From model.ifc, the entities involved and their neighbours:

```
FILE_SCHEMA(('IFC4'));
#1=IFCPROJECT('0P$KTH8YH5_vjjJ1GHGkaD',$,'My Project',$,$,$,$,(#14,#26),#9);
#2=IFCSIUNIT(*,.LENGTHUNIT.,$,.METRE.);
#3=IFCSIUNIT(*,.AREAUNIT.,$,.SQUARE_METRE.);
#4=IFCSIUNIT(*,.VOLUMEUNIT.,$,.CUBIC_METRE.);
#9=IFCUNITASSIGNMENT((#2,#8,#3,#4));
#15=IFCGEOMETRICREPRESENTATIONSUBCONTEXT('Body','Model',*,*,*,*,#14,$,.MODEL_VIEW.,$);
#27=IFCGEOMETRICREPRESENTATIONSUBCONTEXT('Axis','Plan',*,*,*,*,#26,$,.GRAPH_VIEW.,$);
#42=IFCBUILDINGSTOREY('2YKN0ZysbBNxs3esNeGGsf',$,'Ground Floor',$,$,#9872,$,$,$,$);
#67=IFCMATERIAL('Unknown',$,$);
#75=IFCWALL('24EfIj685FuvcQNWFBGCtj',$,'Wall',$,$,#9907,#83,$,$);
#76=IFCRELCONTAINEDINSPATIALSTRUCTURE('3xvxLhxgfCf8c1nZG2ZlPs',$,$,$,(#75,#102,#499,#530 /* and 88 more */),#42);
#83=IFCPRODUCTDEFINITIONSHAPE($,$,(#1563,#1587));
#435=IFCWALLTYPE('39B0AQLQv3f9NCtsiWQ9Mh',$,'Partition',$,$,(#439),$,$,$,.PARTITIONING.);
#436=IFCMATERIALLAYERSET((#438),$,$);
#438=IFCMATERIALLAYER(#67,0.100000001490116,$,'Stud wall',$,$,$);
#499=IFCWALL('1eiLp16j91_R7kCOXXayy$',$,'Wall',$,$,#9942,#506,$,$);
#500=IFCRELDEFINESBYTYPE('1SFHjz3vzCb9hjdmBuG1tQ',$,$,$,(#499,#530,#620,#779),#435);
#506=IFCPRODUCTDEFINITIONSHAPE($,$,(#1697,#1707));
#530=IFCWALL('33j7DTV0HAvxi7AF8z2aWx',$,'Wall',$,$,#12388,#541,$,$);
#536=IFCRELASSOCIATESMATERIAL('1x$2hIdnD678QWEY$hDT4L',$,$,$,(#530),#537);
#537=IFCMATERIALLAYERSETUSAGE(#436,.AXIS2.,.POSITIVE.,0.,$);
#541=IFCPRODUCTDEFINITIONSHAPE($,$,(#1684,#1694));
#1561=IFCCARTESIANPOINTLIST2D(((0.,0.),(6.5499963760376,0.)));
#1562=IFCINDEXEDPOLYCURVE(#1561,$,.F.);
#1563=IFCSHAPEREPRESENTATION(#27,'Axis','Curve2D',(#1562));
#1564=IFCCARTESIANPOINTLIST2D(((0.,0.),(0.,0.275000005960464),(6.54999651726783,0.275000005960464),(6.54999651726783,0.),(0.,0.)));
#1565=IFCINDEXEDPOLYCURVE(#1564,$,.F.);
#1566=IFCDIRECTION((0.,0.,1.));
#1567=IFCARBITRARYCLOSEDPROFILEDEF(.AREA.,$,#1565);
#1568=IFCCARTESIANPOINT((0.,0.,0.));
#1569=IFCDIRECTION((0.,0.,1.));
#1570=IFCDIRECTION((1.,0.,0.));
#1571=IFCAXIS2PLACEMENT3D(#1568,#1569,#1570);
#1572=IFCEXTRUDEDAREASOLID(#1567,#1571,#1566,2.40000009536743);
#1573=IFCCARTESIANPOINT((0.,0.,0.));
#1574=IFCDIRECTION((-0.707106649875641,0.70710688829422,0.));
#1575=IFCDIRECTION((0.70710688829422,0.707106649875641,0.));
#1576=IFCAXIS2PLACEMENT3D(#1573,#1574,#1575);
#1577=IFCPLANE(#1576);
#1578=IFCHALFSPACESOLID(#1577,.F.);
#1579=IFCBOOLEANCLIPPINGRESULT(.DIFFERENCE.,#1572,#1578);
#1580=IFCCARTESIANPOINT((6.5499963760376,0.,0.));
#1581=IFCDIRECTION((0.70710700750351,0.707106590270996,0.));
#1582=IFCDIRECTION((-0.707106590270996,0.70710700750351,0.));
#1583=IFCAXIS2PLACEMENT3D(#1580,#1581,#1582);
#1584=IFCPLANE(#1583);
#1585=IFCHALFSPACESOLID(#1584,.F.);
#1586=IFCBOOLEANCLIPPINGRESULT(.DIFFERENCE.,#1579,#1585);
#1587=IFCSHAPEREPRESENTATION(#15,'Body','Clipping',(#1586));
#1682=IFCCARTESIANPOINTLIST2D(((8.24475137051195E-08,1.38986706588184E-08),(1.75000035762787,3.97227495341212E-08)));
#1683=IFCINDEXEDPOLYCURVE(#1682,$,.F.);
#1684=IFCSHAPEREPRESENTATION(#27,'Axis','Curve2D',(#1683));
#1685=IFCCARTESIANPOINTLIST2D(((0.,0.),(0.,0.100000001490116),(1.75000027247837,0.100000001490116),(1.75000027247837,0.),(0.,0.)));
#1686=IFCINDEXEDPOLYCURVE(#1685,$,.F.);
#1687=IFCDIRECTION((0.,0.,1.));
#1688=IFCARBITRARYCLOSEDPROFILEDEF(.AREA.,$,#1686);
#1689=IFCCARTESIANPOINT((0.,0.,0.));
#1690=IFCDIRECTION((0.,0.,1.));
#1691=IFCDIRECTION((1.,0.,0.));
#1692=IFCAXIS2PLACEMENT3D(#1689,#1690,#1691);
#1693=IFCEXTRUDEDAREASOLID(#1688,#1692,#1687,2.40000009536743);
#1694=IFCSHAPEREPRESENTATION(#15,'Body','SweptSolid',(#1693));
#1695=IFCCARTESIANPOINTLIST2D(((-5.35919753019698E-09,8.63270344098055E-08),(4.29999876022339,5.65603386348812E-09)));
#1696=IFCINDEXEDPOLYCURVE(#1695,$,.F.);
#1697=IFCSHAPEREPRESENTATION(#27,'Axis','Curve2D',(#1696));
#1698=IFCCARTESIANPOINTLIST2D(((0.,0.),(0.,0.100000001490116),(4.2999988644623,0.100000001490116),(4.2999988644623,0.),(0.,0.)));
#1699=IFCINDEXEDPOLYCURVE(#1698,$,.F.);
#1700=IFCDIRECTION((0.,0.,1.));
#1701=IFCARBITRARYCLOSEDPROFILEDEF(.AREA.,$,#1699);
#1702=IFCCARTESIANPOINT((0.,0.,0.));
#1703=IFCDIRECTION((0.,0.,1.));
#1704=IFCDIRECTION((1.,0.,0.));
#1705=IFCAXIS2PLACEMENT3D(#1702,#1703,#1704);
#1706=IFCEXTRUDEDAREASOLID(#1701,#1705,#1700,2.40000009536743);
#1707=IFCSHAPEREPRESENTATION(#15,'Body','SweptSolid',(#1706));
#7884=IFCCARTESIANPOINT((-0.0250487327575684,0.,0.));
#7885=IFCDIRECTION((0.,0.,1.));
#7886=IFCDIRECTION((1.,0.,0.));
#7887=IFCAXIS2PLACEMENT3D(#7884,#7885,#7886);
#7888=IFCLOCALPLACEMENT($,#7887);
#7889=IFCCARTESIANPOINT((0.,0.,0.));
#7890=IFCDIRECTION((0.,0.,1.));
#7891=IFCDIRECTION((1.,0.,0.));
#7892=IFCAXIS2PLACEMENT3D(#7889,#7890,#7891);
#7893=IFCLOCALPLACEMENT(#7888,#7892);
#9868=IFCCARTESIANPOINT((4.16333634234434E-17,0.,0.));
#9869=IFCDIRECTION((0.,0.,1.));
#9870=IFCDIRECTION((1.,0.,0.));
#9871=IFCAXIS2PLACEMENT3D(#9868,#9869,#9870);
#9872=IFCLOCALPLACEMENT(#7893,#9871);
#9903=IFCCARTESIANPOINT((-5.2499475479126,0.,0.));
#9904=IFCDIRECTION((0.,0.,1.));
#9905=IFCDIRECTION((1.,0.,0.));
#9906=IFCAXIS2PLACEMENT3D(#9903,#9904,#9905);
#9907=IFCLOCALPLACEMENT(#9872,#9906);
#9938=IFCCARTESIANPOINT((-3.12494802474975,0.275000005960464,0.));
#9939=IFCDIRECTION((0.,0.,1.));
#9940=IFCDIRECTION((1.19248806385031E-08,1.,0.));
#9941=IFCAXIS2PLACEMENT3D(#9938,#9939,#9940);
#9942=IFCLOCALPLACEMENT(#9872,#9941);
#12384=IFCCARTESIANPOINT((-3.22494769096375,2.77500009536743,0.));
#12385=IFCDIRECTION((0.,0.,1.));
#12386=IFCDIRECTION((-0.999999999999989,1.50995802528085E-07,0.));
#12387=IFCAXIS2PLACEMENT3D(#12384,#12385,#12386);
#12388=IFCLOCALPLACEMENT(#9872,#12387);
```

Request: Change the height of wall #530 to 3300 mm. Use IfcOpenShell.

```python
import ifcopenshell
import ifcopenshell.geom
import ifcopenshell.util.representation
import ifcopenshell.util.shape
import ifcopenshell.util.unit

model = ifcopenshell.open("model.ifc")
unit_scale = ifcopenshell.util.unit.calculate_unit_scale(model)
settings = ifcopenshell.geom.settings()


def volume(element):
    """Net volume in cubic metres, openings subtracted."""
    shape = ifcopenshell.geom.create_shape(settings, element)
    return ifcopenshell.util.shape.get_volume(shape.geometry)


wall = model.by_id(530)
before = volume(wall)

body = ifcopenshell.util.representation.get_representation(wall, "Model", "Body")
solid = body.Items[0]
old_height = solid.Depth
solid.Depth = 3.3 / unit_scale
after = volume(wall)

print(f"height {old_height:g} -> {solid.Depth:g}, volume {before:.3f} -> {after:.3f} m3")

model.write("model_rev.ifc")
```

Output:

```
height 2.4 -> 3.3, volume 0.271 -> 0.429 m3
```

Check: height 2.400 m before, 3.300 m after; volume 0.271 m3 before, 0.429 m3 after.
